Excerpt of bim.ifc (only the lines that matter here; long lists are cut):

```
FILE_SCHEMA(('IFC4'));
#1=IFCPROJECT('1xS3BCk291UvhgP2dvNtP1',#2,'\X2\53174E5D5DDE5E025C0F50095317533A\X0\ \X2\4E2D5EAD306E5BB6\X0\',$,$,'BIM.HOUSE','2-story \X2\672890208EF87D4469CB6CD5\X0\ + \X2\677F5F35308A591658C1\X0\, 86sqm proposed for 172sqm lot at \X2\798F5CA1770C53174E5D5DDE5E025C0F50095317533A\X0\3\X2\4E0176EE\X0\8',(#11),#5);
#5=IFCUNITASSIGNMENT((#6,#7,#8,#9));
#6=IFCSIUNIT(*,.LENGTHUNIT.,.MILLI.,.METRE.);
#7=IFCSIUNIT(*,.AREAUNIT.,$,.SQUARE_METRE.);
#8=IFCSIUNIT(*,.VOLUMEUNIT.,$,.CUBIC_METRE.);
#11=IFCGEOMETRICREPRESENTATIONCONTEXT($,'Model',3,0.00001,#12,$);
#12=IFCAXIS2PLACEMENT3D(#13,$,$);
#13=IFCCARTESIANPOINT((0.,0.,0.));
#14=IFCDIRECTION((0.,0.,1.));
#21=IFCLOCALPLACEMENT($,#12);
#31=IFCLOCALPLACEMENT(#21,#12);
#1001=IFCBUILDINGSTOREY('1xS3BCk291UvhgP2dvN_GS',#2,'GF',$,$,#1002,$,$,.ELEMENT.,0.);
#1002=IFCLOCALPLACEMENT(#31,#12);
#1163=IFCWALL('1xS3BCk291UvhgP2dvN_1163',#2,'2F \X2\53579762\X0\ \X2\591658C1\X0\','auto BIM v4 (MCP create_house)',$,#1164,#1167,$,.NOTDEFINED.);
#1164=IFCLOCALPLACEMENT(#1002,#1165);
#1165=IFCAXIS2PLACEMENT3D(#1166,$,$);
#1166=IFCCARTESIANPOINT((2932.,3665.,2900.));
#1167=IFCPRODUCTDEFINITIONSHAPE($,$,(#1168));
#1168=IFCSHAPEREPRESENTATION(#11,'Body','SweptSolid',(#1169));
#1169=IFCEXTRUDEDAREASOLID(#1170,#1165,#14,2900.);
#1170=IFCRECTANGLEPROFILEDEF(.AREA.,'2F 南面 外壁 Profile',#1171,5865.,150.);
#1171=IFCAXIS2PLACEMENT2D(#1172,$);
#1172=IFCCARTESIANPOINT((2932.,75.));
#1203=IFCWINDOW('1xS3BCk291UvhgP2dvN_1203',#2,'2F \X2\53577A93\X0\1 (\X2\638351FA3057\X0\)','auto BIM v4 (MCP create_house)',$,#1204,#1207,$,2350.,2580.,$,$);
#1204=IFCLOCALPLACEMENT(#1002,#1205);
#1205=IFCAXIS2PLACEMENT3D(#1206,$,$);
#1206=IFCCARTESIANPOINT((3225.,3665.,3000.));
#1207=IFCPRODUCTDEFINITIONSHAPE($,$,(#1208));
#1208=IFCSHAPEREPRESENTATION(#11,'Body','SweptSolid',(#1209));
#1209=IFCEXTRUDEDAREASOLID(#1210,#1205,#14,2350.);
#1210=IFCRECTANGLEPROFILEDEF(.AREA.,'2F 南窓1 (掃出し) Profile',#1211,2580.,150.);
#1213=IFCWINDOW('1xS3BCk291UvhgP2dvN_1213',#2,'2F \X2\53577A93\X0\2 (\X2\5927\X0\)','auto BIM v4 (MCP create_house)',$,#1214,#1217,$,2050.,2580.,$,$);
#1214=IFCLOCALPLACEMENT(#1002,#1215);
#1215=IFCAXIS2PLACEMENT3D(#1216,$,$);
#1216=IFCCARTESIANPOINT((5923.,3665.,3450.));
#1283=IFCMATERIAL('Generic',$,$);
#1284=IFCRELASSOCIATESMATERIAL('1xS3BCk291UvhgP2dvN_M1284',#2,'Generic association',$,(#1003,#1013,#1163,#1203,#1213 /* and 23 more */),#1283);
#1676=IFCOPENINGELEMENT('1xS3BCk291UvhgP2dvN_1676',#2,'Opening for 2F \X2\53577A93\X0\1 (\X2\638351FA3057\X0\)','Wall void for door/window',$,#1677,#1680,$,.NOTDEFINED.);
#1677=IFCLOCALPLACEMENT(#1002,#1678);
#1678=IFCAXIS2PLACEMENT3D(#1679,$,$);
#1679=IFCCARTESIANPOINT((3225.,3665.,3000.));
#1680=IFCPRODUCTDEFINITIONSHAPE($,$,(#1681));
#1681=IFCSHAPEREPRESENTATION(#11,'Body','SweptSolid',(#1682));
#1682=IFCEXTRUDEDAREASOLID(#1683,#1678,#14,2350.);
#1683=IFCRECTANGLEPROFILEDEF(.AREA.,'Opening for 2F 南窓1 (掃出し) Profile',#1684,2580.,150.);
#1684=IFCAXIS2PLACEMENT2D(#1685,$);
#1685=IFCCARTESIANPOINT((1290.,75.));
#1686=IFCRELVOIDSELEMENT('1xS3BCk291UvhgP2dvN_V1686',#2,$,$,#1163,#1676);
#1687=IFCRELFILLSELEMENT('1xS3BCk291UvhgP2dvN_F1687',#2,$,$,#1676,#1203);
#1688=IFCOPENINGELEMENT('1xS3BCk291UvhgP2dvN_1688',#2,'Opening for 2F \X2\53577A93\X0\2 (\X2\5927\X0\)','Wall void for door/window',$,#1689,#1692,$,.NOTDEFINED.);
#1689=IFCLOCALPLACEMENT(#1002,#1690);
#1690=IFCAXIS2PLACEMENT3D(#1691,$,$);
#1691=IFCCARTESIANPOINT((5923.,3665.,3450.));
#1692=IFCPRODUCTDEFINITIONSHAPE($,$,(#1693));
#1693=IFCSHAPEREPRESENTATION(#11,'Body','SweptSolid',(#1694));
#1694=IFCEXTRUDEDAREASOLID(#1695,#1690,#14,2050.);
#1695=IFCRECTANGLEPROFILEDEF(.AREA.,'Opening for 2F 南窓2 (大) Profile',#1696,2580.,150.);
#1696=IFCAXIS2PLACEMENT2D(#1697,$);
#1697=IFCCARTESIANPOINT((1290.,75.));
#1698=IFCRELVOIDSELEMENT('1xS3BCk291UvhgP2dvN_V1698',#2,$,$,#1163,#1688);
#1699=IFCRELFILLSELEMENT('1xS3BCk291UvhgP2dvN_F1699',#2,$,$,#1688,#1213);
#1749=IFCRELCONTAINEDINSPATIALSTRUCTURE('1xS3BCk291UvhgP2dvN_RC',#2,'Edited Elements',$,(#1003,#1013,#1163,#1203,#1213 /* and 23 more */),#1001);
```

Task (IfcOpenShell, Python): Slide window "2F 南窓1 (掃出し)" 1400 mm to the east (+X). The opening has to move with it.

```python
import ifcopenshell
import ifcopenshell.api.geometry
import ifcopenshell.util.placement
import ifcopenshell.util.unit

model = ifcopenshell.open("bim.ifc")
unit_scale = ifcopenshell.util.unit.calculate_unit_scale(model)

window = model.by_guid("1xS3BCk291UvhgP2dvN_1203")
opening = window.FillsVoids[0].RelatingOpeningElement
wall = opening.VoidsElements[0].RelatingBuildingElement

wall_matrix = ifcopenshell.util.placement.get_local_placement(wall.ObjectPlacement)
shift = wall_matrix[:3, 0] * 1.4 / unit_scale
before = ifcopenshell.util.placement.get_local_placement(window.ObjectPlacement)[:3, 3].copy()

# The window is not placed relative to its opening, so move both.
for product in (opening, window):
    matrix = ifcopenshell.util.placement.get_local_placement(product.ObjectPlacement)
    matrix[:3, 3] += shift
    ifcopenshell.api.geometry.edit_object_placement(model, product=product, matrix=matrix, is_si=False)

after = ifcopenshell.util.placement.get_local_placement(window.ObjectPlacement)[:3, 3]
print("window moved by", (after - before).round(3) + 0.0)

model.write("bim_v2.ifc")
```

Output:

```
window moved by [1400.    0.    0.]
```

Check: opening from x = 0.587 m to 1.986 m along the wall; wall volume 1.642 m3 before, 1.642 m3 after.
